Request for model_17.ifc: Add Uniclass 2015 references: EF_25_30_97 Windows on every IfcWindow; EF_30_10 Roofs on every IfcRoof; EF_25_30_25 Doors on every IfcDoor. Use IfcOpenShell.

First a look at what the model holds.

```python
import ifcopenshell

model = ifcopenshell.open("model_17.ifc")
print(model.schema)
print("classifications:", [c.Name for c in model.by_type("IfcClassification")])
for ifc_class in ("IfcDoor", "IfcRoof", "IfcStair", "IfcWall", "IfcWindow"):
    print(ifc_class, len(model.by_type(ifc_class)))
```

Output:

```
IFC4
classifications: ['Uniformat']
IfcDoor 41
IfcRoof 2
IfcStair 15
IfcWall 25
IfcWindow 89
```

```python
import ifcopenshell
import ifcopenshell.api.classification

model = ifcopenshell.open("model_17.ifc")

system = ifcopenshell.api.classification.add_classification(model, classification="Uniclass 2015")

codes = {
    "IfcWindow": ("EF_25_30_97", "Windows"),
    "IfcRoof": ("EF_30_10", "Roofs"),
    "IfcDoor": ("EF_25_30_25", "Doors"),
}
for ifc_class, (code, name) in codes.items():
    products = model.by_type(ifc_class)
    ifcopenshell.api.classification.add_reference(
        model, products=products, classification=system, identification=code, name=name
    )
    print(code, len(products))

model.write("model_17-out.ifc")
```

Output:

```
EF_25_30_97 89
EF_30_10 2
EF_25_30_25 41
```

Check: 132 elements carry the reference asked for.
